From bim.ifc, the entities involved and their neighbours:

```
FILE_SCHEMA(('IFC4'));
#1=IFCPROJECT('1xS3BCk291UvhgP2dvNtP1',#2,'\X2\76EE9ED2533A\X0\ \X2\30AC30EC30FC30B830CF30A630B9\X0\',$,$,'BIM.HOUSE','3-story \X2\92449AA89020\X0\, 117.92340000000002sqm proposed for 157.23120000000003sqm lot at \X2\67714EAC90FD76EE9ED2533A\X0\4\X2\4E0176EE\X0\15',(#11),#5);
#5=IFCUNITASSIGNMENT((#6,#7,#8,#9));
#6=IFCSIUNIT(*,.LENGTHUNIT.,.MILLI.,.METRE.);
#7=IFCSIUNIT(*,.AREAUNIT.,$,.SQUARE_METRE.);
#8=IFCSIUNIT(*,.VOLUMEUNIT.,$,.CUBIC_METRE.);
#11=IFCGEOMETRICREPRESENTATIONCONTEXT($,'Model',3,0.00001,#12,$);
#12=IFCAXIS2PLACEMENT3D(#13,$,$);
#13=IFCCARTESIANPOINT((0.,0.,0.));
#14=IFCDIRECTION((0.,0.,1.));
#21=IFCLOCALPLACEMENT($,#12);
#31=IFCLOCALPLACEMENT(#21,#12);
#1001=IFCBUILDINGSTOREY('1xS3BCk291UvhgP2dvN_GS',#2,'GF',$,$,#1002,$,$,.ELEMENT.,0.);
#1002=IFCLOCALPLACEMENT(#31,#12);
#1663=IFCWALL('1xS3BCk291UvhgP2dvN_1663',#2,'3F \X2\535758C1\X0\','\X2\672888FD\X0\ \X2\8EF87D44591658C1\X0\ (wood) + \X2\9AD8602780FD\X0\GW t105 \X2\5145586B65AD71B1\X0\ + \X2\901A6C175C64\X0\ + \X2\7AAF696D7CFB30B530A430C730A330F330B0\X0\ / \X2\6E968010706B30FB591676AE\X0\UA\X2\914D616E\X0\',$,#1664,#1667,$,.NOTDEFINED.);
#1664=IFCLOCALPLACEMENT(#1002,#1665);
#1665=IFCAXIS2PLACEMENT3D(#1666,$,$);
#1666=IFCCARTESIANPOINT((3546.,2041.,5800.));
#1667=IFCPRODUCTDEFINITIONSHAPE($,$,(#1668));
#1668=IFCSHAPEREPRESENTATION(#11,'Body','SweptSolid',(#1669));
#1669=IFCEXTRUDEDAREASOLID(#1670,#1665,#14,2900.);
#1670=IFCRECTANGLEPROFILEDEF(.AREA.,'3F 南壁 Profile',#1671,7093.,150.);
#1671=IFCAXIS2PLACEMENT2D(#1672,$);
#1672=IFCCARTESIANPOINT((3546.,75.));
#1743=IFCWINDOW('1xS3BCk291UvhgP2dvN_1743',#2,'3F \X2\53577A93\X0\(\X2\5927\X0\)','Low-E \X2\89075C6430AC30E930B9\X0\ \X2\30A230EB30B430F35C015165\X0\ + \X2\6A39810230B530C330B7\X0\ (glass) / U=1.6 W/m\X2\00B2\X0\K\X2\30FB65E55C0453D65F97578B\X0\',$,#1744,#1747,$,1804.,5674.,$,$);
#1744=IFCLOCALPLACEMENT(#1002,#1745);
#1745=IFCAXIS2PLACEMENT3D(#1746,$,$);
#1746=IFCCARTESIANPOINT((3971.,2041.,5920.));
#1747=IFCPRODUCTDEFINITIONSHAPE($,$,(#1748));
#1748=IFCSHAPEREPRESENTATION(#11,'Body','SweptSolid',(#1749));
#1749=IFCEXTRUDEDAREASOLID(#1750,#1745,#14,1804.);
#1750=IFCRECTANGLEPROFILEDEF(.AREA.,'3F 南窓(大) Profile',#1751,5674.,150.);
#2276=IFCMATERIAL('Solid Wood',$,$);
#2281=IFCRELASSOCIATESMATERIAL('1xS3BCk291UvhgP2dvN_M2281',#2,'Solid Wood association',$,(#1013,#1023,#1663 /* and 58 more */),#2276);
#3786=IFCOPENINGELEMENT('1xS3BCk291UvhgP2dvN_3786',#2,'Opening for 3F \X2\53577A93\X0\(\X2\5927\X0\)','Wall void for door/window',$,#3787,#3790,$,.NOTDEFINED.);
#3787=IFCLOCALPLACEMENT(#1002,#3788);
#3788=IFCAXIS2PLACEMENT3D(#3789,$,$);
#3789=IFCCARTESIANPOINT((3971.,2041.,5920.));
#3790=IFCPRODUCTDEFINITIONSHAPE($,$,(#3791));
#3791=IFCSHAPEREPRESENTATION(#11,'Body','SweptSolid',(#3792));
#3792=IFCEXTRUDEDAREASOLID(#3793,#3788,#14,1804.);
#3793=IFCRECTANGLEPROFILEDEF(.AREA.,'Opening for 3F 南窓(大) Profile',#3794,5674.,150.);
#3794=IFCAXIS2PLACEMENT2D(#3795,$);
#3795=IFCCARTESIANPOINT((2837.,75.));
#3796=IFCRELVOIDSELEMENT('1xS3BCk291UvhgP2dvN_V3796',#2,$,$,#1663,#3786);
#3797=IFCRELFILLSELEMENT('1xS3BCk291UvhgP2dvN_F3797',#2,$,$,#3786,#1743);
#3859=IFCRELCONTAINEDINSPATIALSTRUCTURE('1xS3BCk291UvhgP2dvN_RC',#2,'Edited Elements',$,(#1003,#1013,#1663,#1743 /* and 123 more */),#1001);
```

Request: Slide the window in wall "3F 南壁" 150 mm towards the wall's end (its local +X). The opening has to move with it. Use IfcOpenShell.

```python
import ifcopenshell
import ifcopenshell.api.geometry
import ifcopenshell.util.placement
import ifcopenshell.util.unit

model = ifcopenshell.open("bim.ifc")
unit_scale = ifcopenshell.util.unit.calculate_unit_scale(model)

window = model.by_id(1743)
opening = window.FillsVoids[0].RelatingOpeningElement
wall = opening.VoidsElements[0].RelatingBuildingElement

wall_matrix = ifcopenshell.util.placement.get_local_placement(wall.ObjectPlacement)
shift = wall_matrix[:3, 0] * 0.15 / unit_scale
before = ifcopenshell.util.placement.get_local_placement(window.ObjectPlacement)[:3, 3].copy()

# The window is not placed relative to its opening, so move both.
for product in (opening, window):
    matrix = ifcopenshell.util.placement.get_local_placement(product.ObjectPlacement)
    matrix[:3, 3] += shift
    ifcopenshell.api.geometry.edit_object_placement(model, product=product, matrix=matrix, is_si=False)

after = ifcopenshell.util.placement.get_local_placement(window.ObjectPlacement)[:3, 3]
print("window moved by", (after - before).round(3) + 0.0)

model.write("bim-out.ifc")
```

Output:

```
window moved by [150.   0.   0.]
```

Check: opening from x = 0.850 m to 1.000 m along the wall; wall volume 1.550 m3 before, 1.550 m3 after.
